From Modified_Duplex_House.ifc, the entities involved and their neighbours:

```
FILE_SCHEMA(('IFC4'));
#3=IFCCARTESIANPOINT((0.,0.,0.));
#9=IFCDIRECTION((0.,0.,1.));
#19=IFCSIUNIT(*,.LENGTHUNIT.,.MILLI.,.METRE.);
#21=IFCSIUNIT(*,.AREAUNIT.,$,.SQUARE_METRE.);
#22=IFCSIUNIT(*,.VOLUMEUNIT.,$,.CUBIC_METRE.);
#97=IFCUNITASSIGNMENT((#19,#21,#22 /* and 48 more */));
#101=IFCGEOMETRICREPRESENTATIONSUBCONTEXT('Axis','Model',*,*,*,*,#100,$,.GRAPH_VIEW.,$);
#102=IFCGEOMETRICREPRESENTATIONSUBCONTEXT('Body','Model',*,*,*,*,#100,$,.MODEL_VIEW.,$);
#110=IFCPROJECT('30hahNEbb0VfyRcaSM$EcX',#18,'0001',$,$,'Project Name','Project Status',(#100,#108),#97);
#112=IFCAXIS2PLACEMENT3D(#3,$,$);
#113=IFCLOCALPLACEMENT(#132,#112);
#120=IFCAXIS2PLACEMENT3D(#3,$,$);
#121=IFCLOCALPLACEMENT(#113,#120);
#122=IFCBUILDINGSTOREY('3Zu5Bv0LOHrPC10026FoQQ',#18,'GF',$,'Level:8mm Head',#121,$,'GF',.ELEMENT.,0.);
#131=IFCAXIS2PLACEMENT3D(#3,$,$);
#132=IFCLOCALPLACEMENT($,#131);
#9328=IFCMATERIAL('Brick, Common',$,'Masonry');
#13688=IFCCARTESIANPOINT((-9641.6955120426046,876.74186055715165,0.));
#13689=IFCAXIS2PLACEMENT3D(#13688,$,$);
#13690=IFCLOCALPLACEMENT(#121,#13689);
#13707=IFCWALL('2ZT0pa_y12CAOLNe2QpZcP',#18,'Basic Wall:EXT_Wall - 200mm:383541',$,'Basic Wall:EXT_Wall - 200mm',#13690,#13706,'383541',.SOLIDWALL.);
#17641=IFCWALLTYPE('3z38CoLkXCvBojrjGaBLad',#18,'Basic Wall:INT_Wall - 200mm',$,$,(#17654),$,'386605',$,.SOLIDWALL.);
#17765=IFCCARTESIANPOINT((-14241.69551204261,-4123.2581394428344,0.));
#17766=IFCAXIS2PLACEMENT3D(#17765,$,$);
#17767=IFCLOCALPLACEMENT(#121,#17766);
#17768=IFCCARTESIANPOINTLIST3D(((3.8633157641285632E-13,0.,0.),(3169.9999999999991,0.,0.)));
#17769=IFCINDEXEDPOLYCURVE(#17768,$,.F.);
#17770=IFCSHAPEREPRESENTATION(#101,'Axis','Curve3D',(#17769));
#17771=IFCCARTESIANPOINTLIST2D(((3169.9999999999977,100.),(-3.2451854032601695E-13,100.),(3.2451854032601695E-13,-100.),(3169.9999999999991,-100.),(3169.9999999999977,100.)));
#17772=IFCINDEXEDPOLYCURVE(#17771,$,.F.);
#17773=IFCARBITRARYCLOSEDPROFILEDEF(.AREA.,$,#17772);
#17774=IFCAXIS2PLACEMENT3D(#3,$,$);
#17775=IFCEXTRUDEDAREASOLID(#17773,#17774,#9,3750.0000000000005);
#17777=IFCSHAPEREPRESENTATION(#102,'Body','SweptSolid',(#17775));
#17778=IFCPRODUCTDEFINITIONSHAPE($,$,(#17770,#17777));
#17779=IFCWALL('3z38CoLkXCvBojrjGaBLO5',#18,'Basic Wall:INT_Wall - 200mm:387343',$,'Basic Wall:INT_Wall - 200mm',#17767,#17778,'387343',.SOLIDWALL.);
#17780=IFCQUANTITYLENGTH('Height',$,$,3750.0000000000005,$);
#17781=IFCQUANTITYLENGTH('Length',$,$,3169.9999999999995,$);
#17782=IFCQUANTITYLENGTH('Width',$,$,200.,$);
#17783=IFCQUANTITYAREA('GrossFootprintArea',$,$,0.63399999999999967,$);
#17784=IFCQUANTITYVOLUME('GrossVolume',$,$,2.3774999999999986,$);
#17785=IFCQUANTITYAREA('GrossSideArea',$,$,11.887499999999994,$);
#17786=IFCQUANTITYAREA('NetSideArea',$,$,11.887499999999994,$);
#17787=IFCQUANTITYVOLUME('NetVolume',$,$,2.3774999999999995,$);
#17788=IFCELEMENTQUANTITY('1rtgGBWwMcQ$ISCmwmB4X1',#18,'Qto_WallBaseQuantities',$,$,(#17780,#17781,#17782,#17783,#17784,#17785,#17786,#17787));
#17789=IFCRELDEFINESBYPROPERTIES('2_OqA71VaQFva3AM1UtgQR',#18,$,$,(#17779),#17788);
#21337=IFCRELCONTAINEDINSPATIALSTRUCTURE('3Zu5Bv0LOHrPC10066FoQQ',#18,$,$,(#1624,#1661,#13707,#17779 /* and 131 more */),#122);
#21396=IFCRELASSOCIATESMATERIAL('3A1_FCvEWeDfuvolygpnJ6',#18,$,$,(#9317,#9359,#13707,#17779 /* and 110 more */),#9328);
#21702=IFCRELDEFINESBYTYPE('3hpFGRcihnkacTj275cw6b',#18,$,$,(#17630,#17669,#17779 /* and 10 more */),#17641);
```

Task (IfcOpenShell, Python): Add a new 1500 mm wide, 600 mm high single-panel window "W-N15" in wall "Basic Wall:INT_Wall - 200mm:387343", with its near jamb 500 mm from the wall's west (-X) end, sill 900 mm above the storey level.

```python
import numpy as np
import ifcopenshell
import ifcopenshell.api.feature
import ifcopenshell.api.geometry
import ifcopenshell.api.pset
import ifcopenshell.api.root
import ifcopenshell.api.spatial
import ifcopenshell.geom
import ifcopenshell.util.element
import ifcopenshell.util.placement
import ifcopenshell.util.representation
import ifcopenshell.util.shape
import ifcopenshell.util.unit

model = ifcopenshell.open("Modified_Duplex_House.ifc")
unit_scale = ifcopenshell.util.unit.calculate_unit_scale(model)
area_scale = ifcopenshell.util.unit.calculate_unit_scale(model, "AREAUNIT")
volume_scale = ifcopenshell.util.unit.calculate_unit_scale(model, "VOLUMEUNIT")
settings = ifcopenshell.geom.settings()


def volume(element):
    """Net volume in cubic metres, openings subtracted."""
    shape = ifcopenshell.geom.create_shape(settings, element)
    return ifcopenshell.util.shape.get_volume(shape.geometry)


wall = model.by_id(17779)
storey = ifcopenshell.util.element.get_container(wall, ifc_class="IfcBuildingStorey")
context = ifcopenshell.util.representation.get_context(model, "Model", "Body", "MODEL_VIEW")
before = volume(wall)

width, height, from_end, sill = 1.5, 0.6, 0.5, 0.9  # metres

# The wall runs along its own X axis, and the end named is its -X end.
wall_shape = ifcopenshell.geom.create_shape(settings, wall)
x, y, z = ifcopenshell.util.shape.get_vertices(wall_shape.geometry).T
start = x.min() + from_end
face, thickness = float(y.min()), float(y.max() - y.min())
wall_matrix = ifcopenshell.util.placement.get_local_placement(wall.ObjectPlacement)
level = ifcopenshell.util.placement.get_local_placement(storey.ObjectPlacement)[2, 3]


def in_wall(x, y):
    """Placement at x, y metres in the wall's axes, at sill height."""
    matrix = wall_matrix.copy()
    matrix[:, 3] = wall_matrix @ np.array([x / unit_scale, y / unit_scale, 0.0, 1.0])
    matrix[2, 3] = level + sill / unit_scale
    return matrix


# Opening: a box that overshoots both wall faces by 50 mm.
opening = ifcopenshell.api.root.create_entity(model, ifc_class="IfcOpeningElement", predefined_type="OPENING")
box = ifcopenshell.api.geometry.add_wall_representation(
    model, context=context, length=width, height=height, thickness=thickness + 0.1
)
ifcopenshell.api.geometry.assign_representation(model, product=opening, representation=box)
ifcopenshell.api.geometry.edit_object_placement(model, product=opening, matrix=in_wall(start, face - 0.05), is_si=False)
ifcopenshell.api.feature.add_feature(model, feature=opening, element=wall)

window = ifcopenshell.api.root.create_entity(model, ifc_class="IfcWindow", name="W-N15", predefined_type="WINDOW")
window.OverallWidth, window.OverallHeight = width / unit_scale, height / unit_scale
window.PartitioningType = "SINGLE_PANEL"
body = ifcopenshell.api.geometry.add_window_representation(
    model,
    context=context,
    overall_width=window.OverallWidth,
    overall_height=window.OverallHeight,
    partition_type="SINGLE_PANEL",
)
ifcopenshell.api.geometry.assign_representation(model, product=window, representation=body)
ifcopenshell.api.spatial.assign_container(model, products=[window], relating_structure=storey)
ifcopenshell.api.feature.add_filling(model, opening=opening, element=window)

# Centre the window in the wall's thickness.
ifcopenshell.api.geometry.edit_object_placement(model, product=window, matrix=in_wall(start, face), is_si=False)
window_shape = ifcopenshell.geom.create_shape(settings, window)
depth = ifcopenshell.util.shape.get_vertices(window_shape.geometry)[:, 1]
offset = face + thickness / 2 - (depth.min() + depth.max()) / 2
ifcopenshell.api.geometry.edit_object_placement(model, product=window, matrix=in_wall(start, offset), is_si=False)

after = volume(wall)

# Update the wall's stored quantities.
qto = model.by_id(ifcopenshell.util.element.get_pset(wall, "Qto_WallBaseQuantities", should_inherit=False)["id"])
ifcopenshell.api.pset.edit_qto(model, qto=qto, properties={
    "NetSideArea": after / thickness / area_scale,
    "NetVolume": after / volume_scale,
})

print(f"wall volume {before:.3f} -> {after:.3f} m3")

model.write("Modified_Duplex_House_v2.ifc")
```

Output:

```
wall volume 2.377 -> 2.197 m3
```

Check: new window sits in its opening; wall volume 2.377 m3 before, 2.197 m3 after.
